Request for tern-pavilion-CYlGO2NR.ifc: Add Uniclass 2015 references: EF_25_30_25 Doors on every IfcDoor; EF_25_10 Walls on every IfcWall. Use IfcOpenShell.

First a look at what the model holds.

```python
import ifcopenshell

model = ifcopenshell.open("tern-pavilion-CYlGO2NR.ifc")
print(model.schema)
print("classifications:", [c.Name for c in model.by_type("IfcClassification")])
for ifc_class in ("IfcDoor", "IfcRoof", "IfcStair", "IfcWall", "IfcWindow"):
    print(ifc_class, len(model.by_type(ifc_class)))
```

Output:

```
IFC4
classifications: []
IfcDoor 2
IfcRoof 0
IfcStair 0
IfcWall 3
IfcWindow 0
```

```python
import ifcopenshell
import ifcopenshell.api.classification

model = ifcopenshell.open("tern-pavilion-CYlGO2NR.ifc")

system = ifcopenshell.api.classification.add_classification(model, classification="Uniclass 2015")

codes = {
    "IfcDoor": ("EF_25_30_25", "Doors"),
    "IfcWall": ("EF_25_10", "Walls"),
}
for ifc_class, (code, name) in codes.items():
    products = model.by_type(ifc_class)
    ifcopenshell.api.classification.add_reference(
        model, products=products, classification=system, identification=code, name=name
    )
    print(code, len(products))

model.write("tern-pavilion-CYlGO2NR_updated.ifc")
```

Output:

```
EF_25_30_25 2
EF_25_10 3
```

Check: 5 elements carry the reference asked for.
